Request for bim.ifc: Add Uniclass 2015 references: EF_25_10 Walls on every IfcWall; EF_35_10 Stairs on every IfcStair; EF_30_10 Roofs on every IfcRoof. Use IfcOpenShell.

First a look at what the model holds.

```python
import ifcopenshell

model = ifcopenshell.open("bim.ifc")
print(model.schema)
print("classifications:", [c.Name for c in model.by_type("IfcClassification")])
for ifc_class in ("IfcDoor", "IfcRoof", "IfcStair", "IfcWall", "IfcWindow"):
    print(ifc_class, len(model.by_type(ifc_class)))
```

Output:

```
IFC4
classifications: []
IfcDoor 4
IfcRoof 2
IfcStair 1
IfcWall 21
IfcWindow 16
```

```python
import ifcopenshell
import ifcopenshell.api.classification

model = ifcopenshell.open("bim.ifc")

system = ifcopenshell.api.classification.add_classification(model, classification="Uniclass 2015")

codes = {
    "IfcWall": ("EF_25_10", "Walls"),
    "IfcStair": ("EF_35_10", "Stairs"),
    "IfcRoof": ("EF_30_10", "Roofs"),
}
for ifc_class, (code, name) in codes.items():
    products = model.by_type(ifc_class)
    ifcopenshell.api.classification.add_reference(
        model, products=products, classification=system, identification=code, name=name
    )
    print(code, len(products))

model.write("bim_v2.ifc")
```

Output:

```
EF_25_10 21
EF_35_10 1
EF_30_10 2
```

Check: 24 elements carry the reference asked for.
